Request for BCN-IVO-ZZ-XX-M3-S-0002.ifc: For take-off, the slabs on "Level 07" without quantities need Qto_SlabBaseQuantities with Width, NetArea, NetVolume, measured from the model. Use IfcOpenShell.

First a look at what the model holds.

```python
import ifcopenshell
import ifcopenshell.util.element
import ifcopenshell.util.unit

model = ifcopenshell.open("BCN-IVO-ZZ-XX-M3-S-0002.ifc")
print(model.schema)
for unit_type in ("LENGTHUNIT", "AREAUNIT", "VOLUMEUNIT"):
    print(unit_type, ifcopenshell.util.unit.calculate_unit_scale(model, unit_type))
storey = next(s for s in model.by_type("IfcBuildingStorey") if s.Name == "Level 07")
slabs = [e for e in ifcopenshell.util.element.get_decomposition(storey) if e.is_a("IfcSlab")]
for e in sorted(slabs, key=lambda e: e.id()):
    print(e.id(), e.is_a(), e.Name, list(ifcopenshell.util.element.get_psets(e, qtos_only=True)), sep=" | ")
```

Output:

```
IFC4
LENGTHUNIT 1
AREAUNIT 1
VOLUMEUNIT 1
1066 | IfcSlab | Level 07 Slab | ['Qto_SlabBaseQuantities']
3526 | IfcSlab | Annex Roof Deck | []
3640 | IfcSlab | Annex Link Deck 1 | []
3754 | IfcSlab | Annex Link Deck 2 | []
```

```python
import ifcopenshell
import ifcopenshell.api.pset
import ifcopenshell.geom
import ifcopenshell.util.element
import ifcopenshell.util.shape
import ifcopenshell.util.unit

model = ifcopenshell.open("BCN-IVO-ZZ-XX-M3-S-0002.ifc")
unit_scale = ifcopenshell.util.unit.calculate_unit_scale(model)
area_scale = ifcopenshell.util.unit.calculate_unit_scale(model, "AREAUNIT")
volume_scale = ifcopenshell.util.unit.calculate_unit_scale(model, "VOLUMEUNIT")
settings = ifcopenshell.geom.settings()

storey = next(s for s in model.by_type("IfcBuildingStorey") if s.Name == "Level 07")
slabs = [e for e in ifcopenshell.util.element.get_decomposition(storey) if e.is_a("IfcSlab")]

for e in sorted(slabs, key=lambda e: e.id()):
    if ifcopenshell.util.element.get_psets(e, qtos_only=True, should_inherit=False):
        continue
    # Geometry comes back in metres, in the element's own axes.
    shape = ifcopenshell.geom.create_shape(settings, e)
    values = {
        "Width": ifcopenshell.util.shape.get_z(shape.geometry) / unit_scale,
        "NetArea": ifcopenshell.util.shape.get_footprint_area(shape.geometry) / area_scale,
        "NetVolume": ifcopenshell.util.shape.get_volume(shape.geometry) / volume_scale,
    }
    qto = ifcopenshell.api.pset.add_qto(model, product=e, name="Qto_SlabBaseQuantities")
    ifcopenshell.api.pset.edit_qto(model, qto=qto, properties=values)
    print(e.id(), {k: round(v, 3) for k, v in values.items()})

model.write("BCN-IVO-ZZ-XX-M3-S-0002_edited.ifc")
```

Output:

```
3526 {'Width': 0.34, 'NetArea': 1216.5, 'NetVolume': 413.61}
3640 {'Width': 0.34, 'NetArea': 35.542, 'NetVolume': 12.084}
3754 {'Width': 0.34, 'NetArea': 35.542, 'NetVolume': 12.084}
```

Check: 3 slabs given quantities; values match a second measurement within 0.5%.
